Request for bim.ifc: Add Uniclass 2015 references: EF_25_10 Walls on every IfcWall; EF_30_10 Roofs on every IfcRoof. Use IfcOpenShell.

First a look at what the model holds.

```python
import ifcopenshell

model = ifcopenshell.open("bim.ifc")
print(model.schema)
print("classifications:", [c.Name for c in model.by_type("IfcClassification")])
for ifc_class in ("IfcDoor", "IfcRoof", "IfcStair", "IfcWall", "IfcWindow"):
    print(ifc_class, len(model.by_type(ifc_class)))
```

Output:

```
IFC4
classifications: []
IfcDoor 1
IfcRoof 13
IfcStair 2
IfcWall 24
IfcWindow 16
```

```python
import ifcopenshell
import ifcopenshell.api.classification

model = ifcopenshell.open("bim.ifc")

system = ifcopenshell.api.classification.add_classification(model, classification="Uniclass 2015")

codes = {
    "IfcWall": ("EF_25_10", "Walls"),
    "IfcRoof": ("EF_30_10", "Roofs"),
}
for ifc_class, (code, name) in codes.items():
    products = model.by_type(ifc_class)
    ifcopenshell.api.classification.add_reference(
        model, products=products, classification=system, identification=code, name=name
    )
    print(code, len(products))

model.write("bim_updated.ifc")
```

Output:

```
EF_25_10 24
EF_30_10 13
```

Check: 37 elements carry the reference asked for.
